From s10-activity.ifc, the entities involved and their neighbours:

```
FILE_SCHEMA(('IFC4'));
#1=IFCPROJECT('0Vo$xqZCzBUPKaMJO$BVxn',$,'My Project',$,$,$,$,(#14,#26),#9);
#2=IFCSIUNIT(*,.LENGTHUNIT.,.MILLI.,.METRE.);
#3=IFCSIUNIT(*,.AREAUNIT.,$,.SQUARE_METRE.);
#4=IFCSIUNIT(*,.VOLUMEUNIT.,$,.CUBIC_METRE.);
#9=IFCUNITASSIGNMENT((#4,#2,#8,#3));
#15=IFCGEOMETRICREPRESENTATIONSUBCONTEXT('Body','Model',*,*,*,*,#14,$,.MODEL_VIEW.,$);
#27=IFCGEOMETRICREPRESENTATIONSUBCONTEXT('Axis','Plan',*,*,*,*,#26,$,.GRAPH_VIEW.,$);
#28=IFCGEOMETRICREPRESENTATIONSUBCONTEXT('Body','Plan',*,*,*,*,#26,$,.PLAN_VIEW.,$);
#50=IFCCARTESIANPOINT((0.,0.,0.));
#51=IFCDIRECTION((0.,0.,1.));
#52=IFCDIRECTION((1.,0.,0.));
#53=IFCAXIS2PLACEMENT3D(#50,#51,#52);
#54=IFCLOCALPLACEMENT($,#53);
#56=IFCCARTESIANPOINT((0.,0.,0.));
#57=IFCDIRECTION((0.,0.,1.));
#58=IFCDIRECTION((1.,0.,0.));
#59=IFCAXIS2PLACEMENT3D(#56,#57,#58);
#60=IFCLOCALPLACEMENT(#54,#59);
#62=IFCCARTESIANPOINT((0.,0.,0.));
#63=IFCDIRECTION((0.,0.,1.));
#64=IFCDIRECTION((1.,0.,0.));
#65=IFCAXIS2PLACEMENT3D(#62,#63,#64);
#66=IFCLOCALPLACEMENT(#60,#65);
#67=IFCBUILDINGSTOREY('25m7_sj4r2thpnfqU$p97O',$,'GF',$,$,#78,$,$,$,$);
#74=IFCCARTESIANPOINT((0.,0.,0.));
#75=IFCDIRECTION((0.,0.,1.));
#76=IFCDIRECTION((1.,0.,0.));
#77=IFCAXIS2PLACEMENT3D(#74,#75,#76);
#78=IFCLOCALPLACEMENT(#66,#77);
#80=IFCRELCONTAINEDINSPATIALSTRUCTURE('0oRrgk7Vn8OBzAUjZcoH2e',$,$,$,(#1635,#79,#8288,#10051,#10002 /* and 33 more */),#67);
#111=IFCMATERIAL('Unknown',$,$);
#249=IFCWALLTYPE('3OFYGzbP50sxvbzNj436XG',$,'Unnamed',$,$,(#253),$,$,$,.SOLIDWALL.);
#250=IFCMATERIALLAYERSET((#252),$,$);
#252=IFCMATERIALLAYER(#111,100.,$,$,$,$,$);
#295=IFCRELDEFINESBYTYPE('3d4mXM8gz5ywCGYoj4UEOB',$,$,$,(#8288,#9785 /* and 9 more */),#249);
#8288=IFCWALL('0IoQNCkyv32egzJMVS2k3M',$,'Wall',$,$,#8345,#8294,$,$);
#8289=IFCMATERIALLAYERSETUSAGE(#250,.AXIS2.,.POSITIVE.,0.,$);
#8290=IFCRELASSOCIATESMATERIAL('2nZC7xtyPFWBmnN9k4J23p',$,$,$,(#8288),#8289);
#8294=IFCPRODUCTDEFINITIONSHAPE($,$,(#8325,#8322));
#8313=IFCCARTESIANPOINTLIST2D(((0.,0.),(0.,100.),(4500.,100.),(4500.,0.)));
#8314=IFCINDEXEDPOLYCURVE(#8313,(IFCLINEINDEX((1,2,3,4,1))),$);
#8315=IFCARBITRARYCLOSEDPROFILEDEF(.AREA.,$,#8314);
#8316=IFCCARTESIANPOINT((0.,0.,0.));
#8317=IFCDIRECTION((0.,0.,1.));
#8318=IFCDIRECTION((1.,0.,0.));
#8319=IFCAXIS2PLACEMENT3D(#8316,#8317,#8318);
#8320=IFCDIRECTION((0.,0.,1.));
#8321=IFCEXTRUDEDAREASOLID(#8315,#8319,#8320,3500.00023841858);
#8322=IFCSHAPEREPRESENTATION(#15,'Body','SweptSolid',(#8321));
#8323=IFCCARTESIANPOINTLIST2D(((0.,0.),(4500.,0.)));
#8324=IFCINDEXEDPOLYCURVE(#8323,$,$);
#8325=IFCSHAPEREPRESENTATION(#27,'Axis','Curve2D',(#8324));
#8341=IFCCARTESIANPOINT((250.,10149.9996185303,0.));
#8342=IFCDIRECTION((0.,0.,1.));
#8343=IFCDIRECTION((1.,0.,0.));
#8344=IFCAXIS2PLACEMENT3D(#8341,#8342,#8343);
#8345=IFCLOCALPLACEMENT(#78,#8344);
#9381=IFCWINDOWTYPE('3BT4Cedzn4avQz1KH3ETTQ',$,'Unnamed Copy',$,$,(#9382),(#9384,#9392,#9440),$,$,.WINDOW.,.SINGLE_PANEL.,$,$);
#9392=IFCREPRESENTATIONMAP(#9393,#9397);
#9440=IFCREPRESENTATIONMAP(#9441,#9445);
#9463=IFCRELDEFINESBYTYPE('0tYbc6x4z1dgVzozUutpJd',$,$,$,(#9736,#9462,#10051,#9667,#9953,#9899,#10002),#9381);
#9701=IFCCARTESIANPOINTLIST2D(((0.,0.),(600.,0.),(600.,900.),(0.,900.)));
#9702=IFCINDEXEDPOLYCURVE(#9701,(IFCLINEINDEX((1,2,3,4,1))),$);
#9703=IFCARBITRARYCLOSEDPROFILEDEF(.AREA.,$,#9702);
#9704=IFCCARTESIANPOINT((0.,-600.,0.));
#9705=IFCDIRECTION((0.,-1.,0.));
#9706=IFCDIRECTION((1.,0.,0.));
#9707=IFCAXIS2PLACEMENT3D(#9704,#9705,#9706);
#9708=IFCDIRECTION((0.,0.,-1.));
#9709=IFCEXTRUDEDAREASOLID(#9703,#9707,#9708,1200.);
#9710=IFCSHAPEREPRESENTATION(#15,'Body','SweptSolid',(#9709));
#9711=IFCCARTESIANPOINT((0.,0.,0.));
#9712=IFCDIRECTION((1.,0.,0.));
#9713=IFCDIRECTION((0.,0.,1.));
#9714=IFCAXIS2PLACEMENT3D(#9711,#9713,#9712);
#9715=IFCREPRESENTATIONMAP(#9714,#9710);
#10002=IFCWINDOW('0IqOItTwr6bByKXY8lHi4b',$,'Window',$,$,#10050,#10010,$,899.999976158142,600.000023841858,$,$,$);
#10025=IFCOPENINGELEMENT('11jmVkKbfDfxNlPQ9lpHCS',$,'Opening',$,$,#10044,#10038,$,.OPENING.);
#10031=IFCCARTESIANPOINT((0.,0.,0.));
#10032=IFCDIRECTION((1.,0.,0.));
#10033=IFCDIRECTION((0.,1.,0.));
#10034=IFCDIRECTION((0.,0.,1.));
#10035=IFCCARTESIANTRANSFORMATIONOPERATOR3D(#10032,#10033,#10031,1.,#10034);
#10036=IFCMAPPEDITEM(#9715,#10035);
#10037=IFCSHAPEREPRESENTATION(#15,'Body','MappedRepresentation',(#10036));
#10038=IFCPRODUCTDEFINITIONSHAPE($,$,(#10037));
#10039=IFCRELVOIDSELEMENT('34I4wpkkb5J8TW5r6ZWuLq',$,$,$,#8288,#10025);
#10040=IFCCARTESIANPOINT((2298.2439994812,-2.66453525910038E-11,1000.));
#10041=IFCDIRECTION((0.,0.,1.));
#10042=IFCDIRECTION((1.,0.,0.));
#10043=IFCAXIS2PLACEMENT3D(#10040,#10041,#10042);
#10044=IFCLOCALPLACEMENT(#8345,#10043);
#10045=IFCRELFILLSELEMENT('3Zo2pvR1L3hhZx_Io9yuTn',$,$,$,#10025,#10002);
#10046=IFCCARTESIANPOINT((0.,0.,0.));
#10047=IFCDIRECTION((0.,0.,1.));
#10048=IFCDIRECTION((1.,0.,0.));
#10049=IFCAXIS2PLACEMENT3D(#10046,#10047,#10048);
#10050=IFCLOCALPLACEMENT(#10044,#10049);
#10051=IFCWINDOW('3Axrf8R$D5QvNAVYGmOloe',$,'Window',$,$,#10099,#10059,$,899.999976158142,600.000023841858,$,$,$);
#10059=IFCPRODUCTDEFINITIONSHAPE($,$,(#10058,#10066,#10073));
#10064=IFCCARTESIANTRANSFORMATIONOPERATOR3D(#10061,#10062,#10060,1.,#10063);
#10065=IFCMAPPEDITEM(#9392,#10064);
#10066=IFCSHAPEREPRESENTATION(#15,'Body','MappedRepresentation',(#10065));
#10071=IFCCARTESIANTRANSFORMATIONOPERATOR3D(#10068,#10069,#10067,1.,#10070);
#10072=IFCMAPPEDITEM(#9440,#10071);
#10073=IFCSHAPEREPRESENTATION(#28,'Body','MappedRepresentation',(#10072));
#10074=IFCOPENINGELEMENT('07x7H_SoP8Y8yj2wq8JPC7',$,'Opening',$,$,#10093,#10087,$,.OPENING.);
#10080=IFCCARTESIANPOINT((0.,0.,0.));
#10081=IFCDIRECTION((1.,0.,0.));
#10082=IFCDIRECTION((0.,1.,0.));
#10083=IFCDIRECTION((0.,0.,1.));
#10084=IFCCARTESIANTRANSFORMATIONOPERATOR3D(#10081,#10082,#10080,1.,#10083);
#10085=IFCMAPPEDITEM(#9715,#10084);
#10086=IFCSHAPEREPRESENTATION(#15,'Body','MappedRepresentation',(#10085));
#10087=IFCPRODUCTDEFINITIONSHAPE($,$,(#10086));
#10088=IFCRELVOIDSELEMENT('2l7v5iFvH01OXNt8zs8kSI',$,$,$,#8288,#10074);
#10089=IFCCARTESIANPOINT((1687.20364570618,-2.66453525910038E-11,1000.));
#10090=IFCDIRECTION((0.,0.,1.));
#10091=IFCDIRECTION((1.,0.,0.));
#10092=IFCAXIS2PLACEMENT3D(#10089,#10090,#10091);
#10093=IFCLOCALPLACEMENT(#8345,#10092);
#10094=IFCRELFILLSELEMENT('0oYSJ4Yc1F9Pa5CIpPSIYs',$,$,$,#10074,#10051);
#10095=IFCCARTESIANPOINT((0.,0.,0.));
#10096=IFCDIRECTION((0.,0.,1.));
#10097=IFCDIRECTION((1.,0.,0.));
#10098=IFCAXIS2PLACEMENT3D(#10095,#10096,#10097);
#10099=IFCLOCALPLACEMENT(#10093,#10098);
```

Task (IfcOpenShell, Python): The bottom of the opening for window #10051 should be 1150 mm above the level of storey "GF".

```python
import numpy as np
import ifcopenshell
import ifcopenshell.api.geometry
import ifcopenshell.geom
import ifcopenshell.util.element
import ifcopenshell.util.placement
import ifcopenshell.util.shape
import ifcopenshell.util.unit

model = ifcopenshell.open("s10-activity.ifc")
unit_scale = ifcopenshell.util.unit.calculate_unit_scale(model)

window = model.by_guid("3Axrf8R$D5QvNAVYGmOloe")
opening = window.FillsVoids[0].RelatingOpeningElement
storey = ifcopenshell.util.element.get_container(window, ifc_class="IfcBuildingStorey")
level = ifcopenshell.util.placement.get_local_placement(storey.ObjectPlacement)[2, 3]

# The opening's origin need not be at the sill, so measure its lowest point.
shape = ifcopenshell.geom.create_shape(ifcopenshell.geom.settings(), opening)
bottom = ifcopenshell.util.shape.get_shape_bottom_elevation(shape, shape.geometry) / unit_scale
dz = level + 1.15 / unit_scale - bottom

shift = np.array([0.0, 0.0, dz])
# The window is placed relative to its opening, so it follows when the opening moves.
matrix = ifcopenshell.util.placement.get_local_placement(opening.ObjectPlacement)
matrix[:3, 3] += shift
ifcopenshell.api.geometry.edit_object_placement(
    model, product=opening, matrix=matrix, is_si=False, should_transform_children=True
)

print(f"moved by {dz * unit_scale:+.3f} m")

model.write("s10-activity_edited.ifc")
```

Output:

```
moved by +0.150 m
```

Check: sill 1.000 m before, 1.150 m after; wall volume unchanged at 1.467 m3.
